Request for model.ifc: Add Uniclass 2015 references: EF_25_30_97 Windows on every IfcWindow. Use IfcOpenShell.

First a look at what the model holds.

```python
import ifcopenshell

model = ifcopenshell.open("model.ifc")
print(model.schema)
print("classifications:", [c.Name for c in model.by_type("IfcClassification")])
for ifc_class in ("IfcDoor", "IfcRoof", "IfcStair", "IfcWall", "IfcWindow"):
    print(ifc_class, len(model.by_type(ifc_class)))
```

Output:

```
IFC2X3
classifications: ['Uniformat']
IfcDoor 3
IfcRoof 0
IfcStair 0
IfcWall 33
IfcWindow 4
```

```python
import ifcopenshell
import ifcopenshell.api.classification

model = ifcopenshell.open("model.ifc")

# IFC2X3 requires Source and Edition and has no link from the project to the system.
system = model.create_entity("IfcClassification", Source="NBS", Edition="2015", Name="Uniclass 2015")

codes = {
    "IfcWindow": ("EF_25_30_97", "Windows"),
}
for ifc_class, (code, name) in codes.items():
    products = model.by_type(ifc_class)
    ifcopenshell.api.classification.add_reference(
        model, products=products, classification=system, identification=code, name=name
    )
    print(code, len(products))

model.write("model_updated.ifc")
```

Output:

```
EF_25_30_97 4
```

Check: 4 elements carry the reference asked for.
